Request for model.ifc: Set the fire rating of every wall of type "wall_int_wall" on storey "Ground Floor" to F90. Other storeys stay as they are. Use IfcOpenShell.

First a look at what the model holds.

```python
import ifcopenshell
import ifcopenshell.util.element

model = ifcopenshell.open("model.ifc")
print(model.schema)
storey = next(s for s in model.by_type("IfcBuildingStorey") if s.Name == "Ground Floor")
walls = [e for e in ifcopenshell.util.element.get_decomposition(storey) if e.is_a("IfcWall")]
seen = {}
for e in walls:
    element_type = ifcopenshell.util.element.get_type(e)
    key = (element_type.Name if element_type != e and element_type else None, ifcopenshell.util.element.get_pset(e, "Pset_WallCommon", "FireRating"))
    seen[key] = seen.get(key, 0) + 1
for (name, value), count in sorted(seen.items(), key=str):
    print(count, "x", name, "|", value)
```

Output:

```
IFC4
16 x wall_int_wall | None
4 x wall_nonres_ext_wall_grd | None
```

```python
import ifcopenshell
import ifcopenshell.api.pset
import ifcopenshell.util.element

model = ifcopenshell.open("model.ifc")

storey = next(s for s in model.by_type("IfcBuildingStorey") if s.Name == "Ground Floor")
walls = [e for e in ifcopenshell.util.element.get_decomposition(storey) if e.is_a("IfcWall")]

count = 0
for e in walls:
    element_type = ifcopenshell.util.element.get_type(e)
    if element_type in (None, e) or element_type.Name != "wall_int_wall":
        continue
    # add_pset returns the element's existing set when there is one.
    pset = ifcopenshell.api.pset.add_pset(model, product=e, name="Pset_WallCommon")
    ifcopenshell.api.pset.edit_pset(model, pset=pset, properties={"FireRating": "F90"})
    count += 1

print(count, "walls updated")

model.write("model-out.ifc")
```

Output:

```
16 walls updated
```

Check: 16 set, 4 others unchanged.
